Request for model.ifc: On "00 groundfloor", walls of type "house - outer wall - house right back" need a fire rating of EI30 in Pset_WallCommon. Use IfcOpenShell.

First a look at what the model holds.

```python
import ifcopenshell
import ifcopenshell.util.element

model = ifcopenshell.open("model.ifc")
print(model.schema)
storey = next(s for s in model.by_type("IfcBuildingStorey") if s.Name == "00 groundfloor")
walls = [e for e in ifcopenshell.util.element.get_decomposition(storey) if e.is_a("IfcWall")]
seen = {}
for e in walls:
    element_type = ifcopenshell.util.element.get_type(e)
    key = (element_type.Name if element_type != e and element_type else None, ifcopenshell.util.element.get_pset(e, "Pset_WallCommon", "FireRating"))
    seen[key] = seen.get(key, 0) + 1
for (name, value), count in sorted(seen.items(), key=str):
    print(count, "x", name, "|", value)
```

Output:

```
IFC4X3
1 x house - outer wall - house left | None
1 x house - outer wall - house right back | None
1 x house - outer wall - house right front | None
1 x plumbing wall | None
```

```python
import ifcopenshell
import ifcopenshell.api.pset
import ifcopenshell.util.element

model = ifcopenshell.open("model.ifc")

storey = next(s for s in model.by_type("IfcBuildingStorey") if s.Name == "00 groundfloor")
walls = [e for e in ifcopenshell.util.element.get_decomposition(storey) if e.is_a("IfcWall")]

count = 0
for e in walls:
    element_type = ifcopenshell.util.element.get_type(e)
    if element_type in (None, e) or element_type.Name != "house - outer wall - house right back":
        continue
    # add_pset returns the element's existing set when there is one.
    pset = ifcopenshell.api.pset.add_pset(model, product=e, name="Pset_WallCommon")
    ifcopenshell.api.pset.edit_pset(model, pset=pset, properties={"FireRating": "EI30"})
    count += 1

print(count, "walls updated")

model.write("model_edited.ifc")
```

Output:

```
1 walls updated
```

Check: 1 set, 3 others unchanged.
